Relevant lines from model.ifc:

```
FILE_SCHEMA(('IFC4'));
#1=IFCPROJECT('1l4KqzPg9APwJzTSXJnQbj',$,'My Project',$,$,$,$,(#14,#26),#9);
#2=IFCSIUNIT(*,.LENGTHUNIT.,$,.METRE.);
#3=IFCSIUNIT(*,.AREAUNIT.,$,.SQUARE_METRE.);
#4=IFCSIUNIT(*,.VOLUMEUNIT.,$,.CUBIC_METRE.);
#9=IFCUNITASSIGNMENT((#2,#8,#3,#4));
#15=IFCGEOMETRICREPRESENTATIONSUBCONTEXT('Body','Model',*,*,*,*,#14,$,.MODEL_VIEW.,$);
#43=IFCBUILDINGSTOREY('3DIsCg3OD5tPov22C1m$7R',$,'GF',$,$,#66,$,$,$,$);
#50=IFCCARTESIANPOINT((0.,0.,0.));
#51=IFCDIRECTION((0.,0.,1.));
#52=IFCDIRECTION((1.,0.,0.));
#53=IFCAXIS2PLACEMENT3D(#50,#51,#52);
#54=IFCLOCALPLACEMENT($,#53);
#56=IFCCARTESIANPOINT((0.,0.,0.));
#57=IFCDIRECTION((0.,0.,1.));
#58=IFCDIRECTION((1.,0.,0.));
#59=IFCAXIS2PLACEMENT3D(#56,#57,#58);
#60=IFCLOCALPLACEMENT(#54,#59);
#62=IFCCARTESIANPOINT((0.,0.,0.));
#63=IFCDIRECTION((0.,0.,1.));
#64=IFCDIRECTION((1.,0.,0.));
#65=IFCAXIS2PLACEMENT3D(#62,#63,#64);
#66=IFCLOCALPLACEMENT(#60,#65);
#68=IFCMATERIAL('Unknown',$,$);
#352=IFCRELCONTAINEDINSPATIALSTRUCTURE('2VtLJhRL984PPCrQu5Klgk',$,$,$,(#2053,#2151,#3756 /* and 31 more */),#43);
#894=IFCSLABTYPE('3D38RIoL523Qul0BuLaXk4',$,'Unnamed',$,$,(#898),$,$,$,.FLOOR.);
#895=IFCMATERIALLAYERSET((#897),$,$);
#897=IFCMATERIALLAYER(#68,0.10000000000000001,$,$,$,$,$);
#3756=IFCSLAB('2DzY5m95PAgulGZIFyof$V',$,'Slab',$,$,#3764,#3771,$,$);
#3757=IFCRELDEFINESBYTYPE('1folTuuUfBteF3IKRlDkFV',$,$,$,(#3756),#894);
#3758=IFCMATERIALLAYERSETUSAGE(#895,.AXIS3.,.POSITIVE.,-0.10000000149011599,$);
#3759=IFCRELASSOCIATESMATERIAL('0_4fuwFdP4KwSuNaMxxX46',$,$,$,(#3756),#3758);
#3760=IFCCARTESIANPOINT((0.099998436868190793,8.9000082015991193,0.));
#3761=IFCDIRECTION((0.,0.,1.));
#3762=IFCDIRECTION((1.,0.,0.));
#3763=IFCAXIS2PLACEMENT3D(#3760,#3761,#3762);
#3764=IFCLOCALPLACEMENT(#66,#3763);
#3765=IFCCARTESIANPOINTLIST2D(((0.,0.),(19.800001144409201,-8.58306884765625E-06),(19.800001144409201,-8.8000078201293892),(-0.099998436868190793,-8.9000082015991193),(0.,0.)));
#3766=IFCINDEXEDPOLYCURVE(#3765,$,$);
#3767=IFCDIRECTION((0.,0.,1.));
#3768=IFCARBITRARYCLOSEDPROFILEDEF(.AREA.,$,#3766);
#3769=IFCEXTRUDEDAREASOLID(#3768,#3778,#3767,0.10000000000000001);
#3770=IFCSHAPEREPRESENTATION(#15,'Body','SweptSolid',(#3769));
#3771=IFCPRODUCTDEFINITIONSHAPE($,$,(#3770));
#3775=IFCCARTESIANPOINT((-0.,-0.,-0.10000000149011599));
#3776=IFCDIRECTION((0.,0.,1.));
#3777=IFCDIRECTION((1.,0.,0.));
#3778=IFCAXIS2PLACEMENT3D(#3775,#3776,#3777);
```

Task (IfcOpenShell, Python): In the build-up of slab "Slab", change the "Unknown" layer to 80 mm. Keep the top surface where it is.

```python
import ifcopenshell
import ifcopenshell.util.element
import ifcopenshell.util.representation

model = ifcopenshell.open("model.ifc")

layer_set = model.by_id(895)
layer = next(l for l in layer_set.MaterialLayers if l.Material and l.Material.Name == "Unknown")
change = 0.08 - layer.LayerThickness
layer.LayerThickness += change

# Geometry does not follow the layer set by itself.
slabs = [e for e in ifcopenshell.util.element.get_elements_by_material(model, layer_set) if e.is_a("IfcSlab")]
for slab in sorted(slabs, key=lambda e: e.id()):
    body = ifcopenshell.util.representation.get_representation(slab, "Model", "Body")
    solid = body.Items[0]
    old_depth = solid.Depth
    solid.Depth += change
    # Extruded upwards: lower the start of the extrusion so the top stays.
    x, y, z = solid.Position.Location.Coordinates
    solid.Position.Location = model.createIfcCartesianPoint((x, y, z - change))
    print(slab.id(), f"{old_depth:g} -> {solid.Depth:g}")

# The layers are counted up from the underside, which has moved.
for usage in {ifcopenshell.util.element.get_material(slab) for slab in slabs}:
    usage.OffsetFromReferenceLine -= change

model.write("model_edited.ifc")
```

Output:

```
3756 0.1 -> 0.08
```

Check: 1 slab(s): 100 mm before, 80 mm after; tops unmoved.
